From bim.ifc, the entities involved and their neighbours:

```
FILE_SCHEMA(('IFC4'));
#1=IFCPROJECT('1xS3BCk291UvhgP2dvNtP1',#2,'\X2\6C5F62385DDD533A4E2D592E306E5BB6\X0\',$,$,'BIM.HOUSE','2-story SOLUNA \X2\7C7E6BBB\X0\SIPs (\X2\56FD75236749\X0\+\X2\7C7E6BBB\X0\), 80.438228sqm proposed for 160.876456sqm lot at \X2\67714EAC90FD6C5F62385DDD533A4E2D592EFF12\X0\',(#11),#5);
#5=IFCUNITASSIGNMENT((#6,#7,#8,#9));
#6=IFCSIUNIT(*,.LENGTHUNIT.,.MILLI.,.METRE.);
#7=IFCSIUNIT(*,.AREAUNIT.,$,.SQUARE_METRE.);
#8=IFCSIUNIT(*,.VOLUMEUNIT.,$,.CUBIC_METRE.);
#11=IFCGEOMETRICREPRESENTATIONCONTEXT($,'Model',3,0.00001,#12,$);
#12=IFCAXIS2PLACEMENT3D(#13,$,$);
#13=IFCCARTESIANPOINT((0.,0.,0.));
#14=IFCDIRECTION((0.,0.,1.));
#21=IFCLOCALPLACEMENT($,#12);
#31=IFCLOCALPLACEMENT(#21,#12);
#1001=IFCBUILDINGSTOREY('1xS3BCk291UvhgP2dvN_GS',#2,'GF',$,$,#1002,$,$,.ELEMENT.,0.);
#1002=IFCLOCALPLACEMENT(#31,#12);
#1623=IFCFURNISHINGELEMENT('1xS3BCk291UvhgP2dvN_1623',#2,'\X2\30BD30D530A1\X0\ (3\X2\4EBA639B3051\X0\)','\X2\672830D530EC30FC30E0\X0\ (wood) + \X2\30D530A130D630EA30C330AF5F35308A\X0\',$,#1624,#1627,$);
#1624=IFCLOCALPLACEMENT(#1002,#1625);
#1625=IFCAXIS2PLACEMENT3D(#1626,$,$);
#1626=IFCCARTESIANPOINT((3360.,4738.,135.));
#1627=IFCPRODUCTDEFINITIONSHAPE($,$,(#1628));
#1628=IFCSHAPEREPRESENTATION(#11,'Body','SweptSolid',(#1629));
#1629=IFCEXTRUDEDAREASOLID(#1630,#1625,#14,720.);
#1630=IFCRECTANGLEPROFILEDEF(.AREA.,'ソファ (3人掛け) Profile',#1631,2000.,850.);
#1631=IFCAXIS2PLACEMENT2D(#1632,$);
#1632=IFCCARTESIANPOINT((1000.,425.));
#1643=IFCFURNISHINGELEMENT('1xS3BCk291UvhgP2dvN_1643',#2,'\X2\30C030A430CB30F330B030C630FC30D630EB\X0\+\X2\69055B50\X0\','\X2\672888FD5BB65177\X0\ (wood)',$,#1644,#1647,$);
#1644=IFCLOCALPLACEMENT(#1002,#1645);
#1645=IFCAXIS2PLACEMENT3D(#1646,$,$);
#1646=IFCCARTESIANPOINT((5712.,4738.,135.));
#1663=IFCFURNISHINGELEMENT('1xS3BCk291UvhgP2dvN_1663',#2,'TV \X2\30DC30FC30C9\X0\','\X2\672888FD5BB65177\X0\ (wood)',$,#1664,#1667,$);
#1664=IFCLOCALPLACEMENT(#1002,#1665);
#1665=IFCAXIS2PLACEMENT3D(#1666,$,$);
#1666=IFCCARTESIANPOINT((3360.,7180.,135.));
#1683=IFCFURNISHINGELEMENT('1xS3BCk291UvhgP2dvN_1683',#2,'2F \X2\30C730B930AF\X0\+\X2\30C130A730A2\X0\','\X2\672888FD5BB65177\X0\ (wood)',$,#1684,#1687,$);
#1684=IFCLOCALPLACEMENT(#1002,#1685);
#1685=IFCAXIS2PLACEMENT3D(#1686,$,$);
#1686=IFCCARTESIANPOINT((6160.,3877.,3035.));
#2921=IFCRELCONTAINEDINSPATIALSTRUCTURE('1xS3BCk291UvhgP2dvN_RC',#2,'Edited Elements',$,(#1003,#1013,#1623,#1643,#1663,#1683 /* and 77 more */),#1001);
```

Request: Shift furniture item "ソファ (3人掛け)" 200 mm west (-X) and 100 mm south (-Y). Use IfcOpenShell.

```python
import ifcopenshell
import ifcopenshell.api.geometry
import ifcopenshell.util.placement
import ifcopenshell.util.unit

model = ifcopenshell.open("bim.ifc")
unit_scale = ifcopenshell.util.unit.calculate_unit_scale(model)

item = model.by_guid("1xS3BCk291UvhgP2dvN_1623")
matrix = ifcopenshell.util.placement.get_local_placement(item.ObjectPlacement)
matrix[0, 3] -= 0.2 / unit_scale
matrix[1, 3] -= 0.1 / unit_scale
ifcopenshell.api.geometry.edit_object_placement(model, product=item, matrix=matrix, is_si=False)

print(ifcopenshell.util.placement.get_local_placement(item.ObjectPlacement).round(3) + 0.0)

model.write("bim_edited.ifc")
```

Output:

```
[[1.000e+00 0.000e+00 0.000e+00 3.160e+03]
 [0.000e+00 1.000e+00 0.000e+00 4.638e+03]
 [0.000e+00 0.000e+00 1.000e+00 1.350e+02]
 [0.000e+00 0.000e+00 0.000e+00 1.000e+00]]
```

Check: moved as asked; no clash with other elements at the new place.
